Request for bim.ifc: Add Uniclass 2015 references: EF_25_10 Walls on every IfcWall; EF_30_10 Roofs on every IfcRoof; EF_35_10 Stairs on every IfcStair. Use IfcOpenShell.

First a look at what the model holds.

```python
import ifcopenshell

model = ifcopenshell.open("bim.ifc")
print(model.schema)
print("classifications:", [c.Name for c in model.by_type("IfcClassification")])
for ifc_class in ("IfcDoor", "IfcRoof", "IfcStair", "IfcWall", "IfcWindow"):
    print(ifc_class, len(model.by_type(ifc_class)))
```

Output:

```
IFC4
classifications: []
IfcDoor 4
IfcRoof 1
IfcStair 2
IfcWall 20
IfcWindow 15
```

```python
import ifcopenshell
import ifcopenshell.api.classification

model = ifcopenshell.open("bim.ifc")

system = ifcopenshell.api.classification.add_classification(model, classification="Uniclass 2015")

codes = {
    "IfcWall": ("EF_25_10", "Walls"),
    "IfcRoof": ("EF_30_10", "Roofs"),
    "IfcStair": ("EF_35_10", "Stairs"),
}
for ifc_class, (code, name) in codes.items():
    products = model.by_type(ifc_class)
    ifcopenshell.api.classification.add_reference(
        model, products=products, classification=system, identification=code, name=name
    )
    print(code, len(products))

model.write("bim_updated.ifc")
```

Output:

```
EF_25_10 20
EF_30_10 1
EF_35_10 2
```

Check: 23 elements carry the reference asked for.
